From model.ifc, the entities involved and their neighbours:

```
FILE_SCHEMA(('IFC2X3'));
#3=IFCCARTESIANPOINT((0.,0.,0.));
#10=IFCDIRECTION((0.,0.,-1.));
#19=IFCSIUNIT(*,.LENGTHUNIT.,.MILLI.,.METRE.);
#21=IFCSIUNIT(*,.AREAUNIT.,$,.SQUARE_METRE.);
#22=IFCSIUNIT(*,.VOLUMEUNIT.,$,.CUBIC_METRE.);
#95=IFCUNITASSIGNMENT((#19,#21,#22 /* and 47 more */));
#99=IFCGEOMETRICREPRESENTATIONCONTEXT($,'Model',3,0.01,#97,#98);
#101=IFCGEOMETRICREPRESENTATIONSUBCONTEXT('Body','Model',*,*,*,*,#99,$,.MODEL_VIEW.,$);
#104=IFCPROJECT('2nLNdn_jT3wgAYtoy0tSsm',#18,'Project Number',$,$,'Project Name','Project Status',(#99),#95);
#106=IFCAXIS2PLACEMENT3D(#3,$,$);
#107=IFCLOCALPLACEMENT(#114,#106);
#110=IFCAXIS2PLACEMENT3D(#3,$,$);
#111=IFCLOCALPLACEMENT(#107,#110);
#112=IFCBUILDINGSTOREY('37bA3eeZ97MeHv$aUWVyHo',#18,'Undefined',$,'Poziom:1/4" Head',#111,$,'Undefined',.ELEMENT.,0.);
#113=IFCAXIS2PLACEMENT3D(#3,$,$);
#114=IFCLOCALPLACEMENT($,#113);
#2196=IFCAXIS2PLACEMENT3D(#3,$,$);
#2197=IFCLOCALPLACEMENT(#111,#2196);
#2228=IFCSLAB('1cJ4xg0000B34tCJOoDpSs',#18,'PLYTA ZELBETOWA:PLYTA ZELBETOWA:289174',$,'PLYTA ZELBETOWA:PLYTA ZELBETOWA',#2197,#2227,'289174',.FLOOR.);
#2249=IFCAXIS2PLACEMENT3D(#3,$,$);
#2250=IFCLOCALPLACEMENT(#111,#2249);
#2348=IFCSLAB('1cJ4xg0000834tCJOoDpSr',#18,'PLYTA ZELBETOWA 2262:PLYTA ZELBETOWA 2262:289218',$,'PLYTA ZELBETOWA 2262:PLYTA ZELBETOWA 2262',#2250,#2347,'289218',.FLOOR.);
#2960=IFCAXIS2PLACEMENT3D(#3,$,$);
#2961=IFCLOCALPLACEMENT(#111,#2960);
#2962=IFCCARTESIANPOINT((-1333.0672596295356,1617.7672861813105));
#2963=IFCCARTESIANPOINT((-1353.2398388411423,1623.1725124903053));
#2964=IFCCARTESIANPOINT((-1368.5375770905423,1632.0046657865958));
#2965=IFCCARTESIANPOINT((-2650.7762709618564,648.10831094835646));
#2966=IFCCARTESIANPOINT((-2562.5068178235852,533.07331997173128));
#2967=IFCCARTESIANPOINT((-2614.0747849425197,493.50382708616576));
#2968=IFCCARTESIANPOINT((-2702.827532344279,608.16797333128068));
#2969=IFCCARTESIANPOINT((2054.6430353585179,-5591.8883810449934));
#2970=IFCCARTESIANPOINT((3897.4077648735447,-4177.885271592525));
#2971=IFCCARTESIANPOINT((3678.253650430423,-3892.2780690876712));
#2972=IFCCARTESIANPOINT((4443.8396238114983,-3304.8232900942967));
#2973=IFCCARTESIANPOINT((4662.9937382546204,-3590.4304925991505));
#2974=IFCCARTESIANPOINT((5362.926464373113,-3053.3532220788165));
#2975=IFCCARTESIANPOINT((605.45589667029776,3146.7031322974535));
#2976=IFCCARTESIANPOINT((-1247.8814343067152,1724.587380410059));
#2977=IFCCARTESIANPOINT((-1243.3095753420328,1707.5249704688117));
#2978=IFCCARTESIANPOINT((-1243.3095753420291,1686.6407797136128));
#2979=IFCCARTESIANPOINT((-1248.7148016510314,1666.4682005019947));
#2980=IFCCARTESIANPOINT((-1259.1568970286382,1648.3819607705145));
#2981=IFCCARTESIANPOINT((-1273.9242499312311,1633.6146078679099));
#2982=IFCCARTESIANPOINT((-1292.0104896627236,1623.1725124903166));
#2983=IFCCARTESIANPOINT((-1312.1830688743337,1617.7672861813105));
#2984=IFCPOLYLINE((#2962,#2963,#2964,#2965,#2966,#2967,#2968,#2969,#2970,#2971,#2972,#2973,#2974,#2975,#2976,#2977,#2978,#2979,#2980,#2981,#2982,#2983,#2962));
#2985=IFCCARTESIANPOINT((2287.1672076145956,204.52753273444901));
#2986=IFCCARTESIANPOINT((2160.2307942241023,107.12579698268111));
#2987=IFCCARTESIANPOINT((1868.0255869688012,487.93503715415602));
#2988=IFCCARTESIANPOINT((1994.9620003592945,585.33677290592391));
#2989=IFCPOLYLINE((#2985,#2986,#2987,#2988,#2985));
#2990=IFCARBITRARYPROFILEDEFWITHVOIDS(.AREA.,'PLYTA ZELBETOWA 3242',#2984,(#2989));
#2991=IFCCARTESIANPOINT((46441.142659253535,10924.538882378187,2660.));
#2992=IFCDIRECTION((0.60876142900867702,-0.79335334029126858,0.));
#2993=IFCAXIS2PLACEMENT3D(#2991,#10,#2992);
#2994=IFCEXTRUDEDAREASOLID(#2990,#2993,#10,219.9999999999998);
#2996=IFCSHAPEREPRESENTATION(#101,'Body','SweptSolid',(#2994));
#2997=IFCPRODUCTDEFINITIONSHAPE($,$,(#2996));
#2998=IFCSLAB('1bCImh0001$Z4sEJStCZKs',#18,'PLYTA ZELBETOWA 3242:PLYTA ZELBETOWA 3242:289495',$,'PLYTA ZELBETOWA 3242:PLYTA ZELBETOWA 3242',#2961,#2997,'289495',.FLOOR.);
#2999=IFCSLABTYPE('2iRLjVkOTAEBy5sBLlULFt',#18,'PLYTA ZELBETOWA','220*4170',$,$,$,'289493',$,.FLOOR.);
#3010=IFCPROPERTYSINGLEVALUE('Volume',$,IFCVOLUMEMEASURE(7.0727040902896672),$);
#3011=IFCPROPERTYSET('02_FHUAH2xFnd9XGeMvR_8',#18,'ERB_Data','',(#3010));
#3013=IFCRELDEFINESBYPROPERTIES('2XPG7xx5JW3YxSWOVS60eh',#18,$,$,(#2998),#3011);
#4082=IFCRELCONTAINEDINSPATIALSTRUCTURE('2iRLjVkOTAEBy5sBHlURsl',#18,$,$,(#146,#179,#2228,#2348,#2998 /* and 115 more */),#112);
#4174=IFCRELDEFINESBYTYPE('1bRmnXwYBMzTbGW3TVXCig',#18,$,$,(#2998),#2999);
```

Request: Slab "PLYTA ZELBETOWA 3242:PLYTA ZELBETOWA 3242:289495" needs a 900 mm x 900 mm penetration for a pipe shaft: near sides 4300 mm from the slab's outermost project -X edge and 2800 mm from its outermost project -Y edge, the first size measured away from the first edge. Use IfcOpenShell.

```python
import numpy as np
import ifcopenshell
import ifcopenshell.api.feature
import ifcopenshell.api.geometry
import ifcopenshell.api.pset
import ifcopenshell.api.root
import ifcopenshell.geom
import ifcopenshell.util.element
import ifcopenshell.util.placement
import ifcopenshell.util.representation
import ifcopenshell.util.shape
import ifcopenshell.util.unit

model = ifcopenshell.open("model.ifc")
unit_scale = ifcopenshell.util.unit.calculate_unit_scale(model)
volume_scale = ifcopenshell.util.unit.calculate_unit_scale(model, "VOLUMEUNIT")
settings = ifcopenshell.geom.settings()


def volume(element):
    """Net volume in cubic metres, openings subtracted."""
    shape = ifcopenshell.geom.create_shape(settings, element)
    return ifcopenshell.util.shape.get_volume(shape.geometry)


slab = model.by_guid("1bCImh0001$Z4sEJStCZKs")
before = volume(slab)

# Extent in the slab's own axes, in metres. The edges named are its -X and -Y sides.
slab_shape = ifcopenshell.geom.create_shape(settings, slab)
vertices = ifcopenshell.util.shape.get_vertices(slab_shape.geometry)
x_min, y_min, bottom = vertices.min(axis=0)
top = vertices[:, 2].max()

opening = ifcopenshell.api.root.create_entity(model, ifc_class="IfcOpeningElement", name="Pipe shaft opening")
context = ifcopenshell.util.representation.get_context(model, "Model", "Body", "MODEL_VIEW")
width, depth = 0.9, 0.9
outline = [(0.0, 0.0), (width, 0.0), (width, depth), (0.0, depth), (0.0, 0.0)]
# Overshoot both faces by 50 mm so the cut is clean.
shape = ifcopenshell.api.geometry.add_slab_representation(
    model, context=context, depth=top - bottom + 0.1, polyline=outline
)
ifcopenshell.api.geometry.assign_representation(model, product=opening, representation=shape)

matrix = ifcopenshell.util.placement.get_local_placement(slab.ObjectPlacement)
matrix[:, 3] = matrix @ np.append(np.array([x_min + 4.3, y_min + 2.8, bottom - 0.05]) / unit_scale, 1.0)
ifcopenshell.api.geometry.edit_object_placement(model, product=opening, matrix=matrix, is_si=False)
ifcopenshell.api.feature.add_feature(model, feature=opening, element=slab)

after = volume(slab)

# Update the slab's stored quantities.
pset = model.by_id(ifcopenshell.util.element.get_pset(slab, "ERB_Data", should_inherit=False)["id"])
ifcopenshell.api.pset.edit_pset(model, pset=pset, properties={
    "Volume": model.create_entity("IfcVolumeMeasure", after / volume_scale),
})

print(f"slab volume {before:.3f} -> {after:.3f} m3")

model.write("model_updated.ifc")
```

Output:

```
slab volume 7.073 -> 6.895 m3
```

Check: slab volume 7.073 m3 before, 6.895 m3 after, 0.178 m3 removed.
